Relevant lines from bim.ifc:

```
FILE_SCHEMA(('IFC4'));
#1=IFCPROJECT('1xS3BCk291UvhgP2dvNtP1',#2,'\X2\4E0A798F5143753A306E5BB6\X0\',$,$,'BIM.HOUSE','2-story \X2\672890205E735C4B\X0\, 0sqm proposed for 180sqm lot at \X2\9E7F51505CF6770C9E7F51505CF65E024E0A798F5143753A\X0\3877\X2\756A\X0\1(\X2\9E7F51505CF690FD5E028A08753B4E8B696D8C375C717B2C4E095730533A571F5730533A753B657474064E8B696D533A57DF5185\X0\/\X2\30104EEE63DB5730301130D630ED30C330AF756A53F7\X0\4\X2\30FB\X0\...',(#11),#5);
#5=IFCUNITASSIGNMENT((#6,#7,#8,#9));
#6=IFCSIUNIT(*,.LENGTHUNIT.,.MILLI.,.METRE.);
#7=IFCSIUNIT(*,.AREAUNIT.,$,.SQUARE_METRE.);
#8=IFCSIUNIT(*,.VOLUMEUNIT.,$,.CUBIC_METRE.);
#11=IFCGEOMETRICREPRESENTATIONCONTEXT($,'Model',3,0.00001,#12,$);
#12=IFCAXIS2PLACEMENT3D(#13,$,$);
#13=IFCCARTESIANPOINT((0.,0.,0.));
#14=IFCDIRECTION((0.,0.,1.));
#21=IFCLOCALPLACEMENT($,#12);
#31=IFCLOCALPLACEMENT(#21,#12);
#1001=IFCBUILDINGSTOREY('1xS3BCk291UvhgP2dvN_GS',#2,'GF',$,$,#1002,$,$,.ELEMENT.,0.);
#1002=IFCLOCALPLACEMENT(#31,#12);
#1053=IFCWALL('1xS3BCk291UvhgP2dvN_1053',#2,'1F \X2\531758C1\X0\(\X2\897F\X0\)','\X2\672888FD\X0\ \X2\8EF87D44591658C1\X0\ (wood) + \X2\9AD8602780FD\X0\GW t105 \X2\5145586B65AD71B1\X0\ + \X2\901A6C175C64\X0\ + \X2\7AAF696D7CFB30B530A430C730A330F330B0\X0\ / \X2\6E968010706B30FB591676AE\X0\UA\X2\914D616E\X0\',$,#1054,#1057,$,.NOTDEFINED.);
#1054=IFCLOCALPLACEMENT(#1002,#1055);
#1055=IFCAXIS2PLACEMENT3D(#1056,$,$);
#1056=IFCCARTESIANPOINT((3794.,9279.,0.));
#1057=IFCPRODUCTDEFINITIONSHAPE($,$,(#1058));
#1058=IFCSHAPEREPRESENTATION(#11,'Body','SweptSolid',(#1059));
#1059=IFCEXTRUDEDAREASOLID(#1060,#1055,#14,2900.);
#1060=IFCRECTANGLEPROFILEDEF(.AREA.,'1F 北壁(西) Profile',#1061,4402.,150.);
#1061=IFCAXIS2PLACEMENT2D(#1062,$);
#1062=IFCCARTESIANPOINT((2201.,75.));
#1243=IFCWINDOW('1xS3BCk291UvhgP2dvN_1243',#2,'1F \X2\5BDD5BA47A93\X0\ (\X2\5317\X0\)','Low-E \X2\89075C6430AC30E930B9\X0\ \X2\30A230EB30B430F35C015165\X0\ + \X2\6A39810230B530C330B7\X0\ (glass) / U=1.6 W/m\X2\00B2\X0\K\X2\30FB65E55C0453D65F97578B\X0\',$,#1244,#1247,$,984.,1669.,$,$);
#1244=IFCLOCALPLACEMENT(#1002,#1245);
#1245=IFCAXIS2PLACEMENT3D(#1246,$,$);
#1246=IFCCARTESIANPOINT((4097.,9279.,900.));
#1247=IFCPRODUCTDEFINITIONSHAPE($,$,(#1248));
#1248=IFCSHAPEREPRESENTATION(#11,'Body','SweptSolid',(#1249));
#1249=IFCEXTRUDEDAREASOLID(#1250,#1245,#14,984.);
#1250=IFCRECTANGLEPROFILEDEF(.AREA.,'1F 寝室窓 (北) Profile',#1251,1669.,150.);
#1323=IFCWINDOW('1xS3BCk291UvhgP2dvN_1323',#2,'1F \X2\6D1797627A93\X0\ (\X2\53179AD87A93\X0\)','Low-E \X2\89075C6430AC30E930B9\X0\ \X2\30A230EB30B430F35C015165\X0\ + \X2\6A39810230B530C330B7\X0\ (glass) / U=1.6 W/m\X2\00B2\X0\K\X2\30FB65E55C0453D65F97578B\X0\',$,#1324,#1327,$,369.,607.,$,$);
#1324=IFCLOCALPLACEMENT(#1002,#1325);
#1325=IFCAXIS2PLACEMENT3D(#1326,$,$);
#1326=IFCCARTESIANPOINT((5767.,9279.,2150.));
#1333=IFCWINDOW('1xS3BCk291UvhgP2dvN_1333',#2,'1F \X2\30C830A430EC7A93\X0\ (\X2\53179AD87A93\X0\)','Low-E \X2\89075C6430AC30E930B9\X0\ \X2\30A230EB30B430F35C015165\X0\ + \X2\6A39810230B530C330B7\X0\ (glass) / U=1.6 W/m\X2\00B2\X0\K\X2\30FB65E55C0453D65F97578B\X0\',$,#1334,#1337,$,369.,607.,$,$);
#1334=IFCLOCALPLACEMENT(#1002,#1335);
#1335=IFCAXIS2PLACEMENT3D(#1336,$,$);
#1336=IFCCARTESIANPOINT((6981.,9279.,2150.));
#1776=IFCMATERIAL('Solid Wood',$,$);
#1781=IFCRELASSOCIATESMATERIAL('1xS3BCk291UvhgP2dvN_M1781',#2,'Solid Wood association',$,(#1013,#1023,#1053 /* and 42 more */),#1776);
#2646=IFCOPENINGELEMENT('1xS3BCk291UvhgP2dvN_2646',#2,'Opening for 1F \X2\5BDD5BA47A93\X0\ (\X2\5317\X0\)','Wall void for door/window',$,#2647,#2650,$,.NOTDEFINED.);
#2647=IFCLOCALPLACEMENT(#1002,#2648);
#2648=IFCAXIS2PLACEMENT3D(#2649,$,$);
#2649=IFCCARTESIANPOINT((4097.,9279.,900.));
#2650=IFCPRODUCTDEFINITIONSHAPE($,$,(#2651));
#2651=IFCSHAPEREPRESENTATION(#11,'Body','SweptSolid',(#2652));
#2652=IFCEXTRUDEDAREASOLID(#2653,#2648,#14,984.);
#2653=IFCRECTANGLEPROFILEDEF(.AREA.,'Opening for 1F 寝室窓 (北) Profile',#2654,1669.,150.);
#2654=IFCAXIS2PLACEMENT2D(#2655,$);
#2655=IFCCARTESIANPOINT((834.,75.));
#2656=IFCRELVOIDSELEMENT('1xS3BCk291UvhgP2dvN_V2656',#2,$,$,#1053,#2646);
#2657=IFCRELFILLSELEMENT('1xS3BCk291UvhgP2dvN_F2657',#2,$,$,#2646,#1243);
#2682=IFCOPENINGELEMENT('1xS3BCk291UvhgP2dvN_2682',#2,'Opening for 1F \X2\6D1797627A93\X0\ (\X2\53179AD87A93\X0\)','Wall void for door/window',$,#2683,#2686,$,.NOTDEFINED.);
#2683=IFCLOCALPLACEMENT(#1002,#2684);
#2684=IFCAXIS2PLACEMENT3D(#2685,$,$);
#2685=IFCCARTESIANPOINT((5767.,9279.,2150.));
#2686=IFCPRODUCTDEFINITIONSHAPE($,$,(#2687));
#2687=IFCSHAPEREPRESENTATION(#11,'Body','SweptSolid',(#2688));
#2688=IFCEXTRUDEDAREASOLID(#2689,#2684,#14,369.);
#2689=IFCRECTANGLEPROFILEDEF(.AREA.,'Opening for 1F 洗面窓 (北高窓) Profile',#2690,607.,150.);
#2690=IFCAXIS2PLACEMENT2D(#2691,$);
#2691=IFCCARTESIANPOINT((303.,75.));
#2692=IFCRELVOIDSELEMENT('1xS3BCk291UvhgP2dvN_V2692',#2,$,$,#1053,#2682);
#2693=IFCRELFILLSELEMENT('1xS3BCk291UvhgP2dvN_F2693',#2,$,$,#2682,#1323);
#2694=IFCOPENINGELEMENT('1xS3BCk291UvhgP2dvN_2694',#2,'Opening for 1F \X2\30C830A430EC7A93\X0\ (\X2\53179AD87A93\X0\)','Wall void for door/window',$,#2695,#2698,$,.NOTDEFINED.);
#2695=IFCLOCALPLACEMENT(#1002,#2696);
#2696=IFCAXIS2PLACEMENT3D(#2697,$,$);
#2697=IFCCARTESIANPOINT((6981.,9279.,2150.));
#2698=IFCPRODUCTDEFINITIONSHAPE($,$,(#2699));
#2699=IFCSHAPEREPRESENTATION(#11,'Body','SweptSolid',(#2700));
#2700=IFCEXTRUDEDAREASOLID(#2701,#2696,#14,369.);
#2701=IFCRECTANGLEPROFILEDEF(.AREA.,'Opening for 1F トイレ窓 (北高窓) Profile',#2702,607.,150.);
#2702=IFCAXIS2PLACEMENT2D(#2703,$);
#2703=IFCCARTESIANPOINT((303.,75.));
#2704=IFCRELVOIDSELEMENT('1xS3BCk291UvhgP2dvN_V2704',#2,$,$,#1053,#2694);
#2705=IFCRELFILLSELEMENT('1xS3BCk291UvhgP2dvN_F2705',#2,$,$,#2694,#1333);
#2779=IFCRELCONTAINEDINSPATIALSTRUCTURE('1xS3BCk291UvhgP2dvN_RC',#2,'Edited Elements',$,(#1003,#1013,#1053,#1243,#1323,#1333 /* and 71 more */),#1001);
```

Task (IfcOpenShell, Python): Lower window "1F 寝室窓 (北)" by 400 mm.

```python
import numpy as np
import ifcopenshell
import ifcopenshell.api.geometry
import ifcopenshell.util.placement
import ifcopenshell.util.unit

model = ifcopenshell.open("bim.ifc")
unit_scale = ifcopenshell.util.unit.calculate_unit_scale(model)

window = model.by_id(1243)
opening = window.FillsVoids[0].RelatingOpeningElement
dz = -400.0

shift = np.array([0.0, 0.0, dz])
# The window is not placed relative to its opening, so move both.
for product in (opening, window):
    matrix = ifcopenshell.util.placement.get_local_placement(product.ObjectPlacement)
    matrix[:3, 3] += shift
    ifcopenshell.api.geometry.edit_object_placement(model, product=product, matrix=matrix, is_si=False)

print(f"moved by {dz * unit_scale:+.3f} m")

model.write("bim-out.ifc")
```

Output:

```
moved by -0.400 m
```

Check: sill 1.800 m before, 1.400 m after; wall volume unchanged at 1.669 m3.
